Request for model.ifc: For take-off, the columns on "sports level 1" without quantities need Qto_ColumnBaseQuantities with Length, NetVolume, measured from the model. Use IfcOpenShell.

First a look at what the model holds.

```python
import ifcopenshell
import ifcopenshell.util.element
import ifcopenshell.util.unit

model = ifcopenshell.open("model.ifc")
print(model.schema)
for unit_type in ("LENGTHUNIT", "AREAUNIT", "VOLUMEUNIT"):
    print(unit_type, ifcopenshell.util.unit.calculate_unit_scale(model, unit_type))
storey = next(s for s in model.by_type("IfcBuildingStorey") if s.Name == "sports level 1")
columns = [e for e in ifcopenshell.util.element.get_decomposition(storey) if e.is_a("IfcColumn")]
for e in sorted(columns, key=lambda e: e.id()):
    print(e.id(), e.is_a(), e.Name, list(ifcopenshell.util.element.get_psets(e, qtos_only=True)), sep=" | ")
```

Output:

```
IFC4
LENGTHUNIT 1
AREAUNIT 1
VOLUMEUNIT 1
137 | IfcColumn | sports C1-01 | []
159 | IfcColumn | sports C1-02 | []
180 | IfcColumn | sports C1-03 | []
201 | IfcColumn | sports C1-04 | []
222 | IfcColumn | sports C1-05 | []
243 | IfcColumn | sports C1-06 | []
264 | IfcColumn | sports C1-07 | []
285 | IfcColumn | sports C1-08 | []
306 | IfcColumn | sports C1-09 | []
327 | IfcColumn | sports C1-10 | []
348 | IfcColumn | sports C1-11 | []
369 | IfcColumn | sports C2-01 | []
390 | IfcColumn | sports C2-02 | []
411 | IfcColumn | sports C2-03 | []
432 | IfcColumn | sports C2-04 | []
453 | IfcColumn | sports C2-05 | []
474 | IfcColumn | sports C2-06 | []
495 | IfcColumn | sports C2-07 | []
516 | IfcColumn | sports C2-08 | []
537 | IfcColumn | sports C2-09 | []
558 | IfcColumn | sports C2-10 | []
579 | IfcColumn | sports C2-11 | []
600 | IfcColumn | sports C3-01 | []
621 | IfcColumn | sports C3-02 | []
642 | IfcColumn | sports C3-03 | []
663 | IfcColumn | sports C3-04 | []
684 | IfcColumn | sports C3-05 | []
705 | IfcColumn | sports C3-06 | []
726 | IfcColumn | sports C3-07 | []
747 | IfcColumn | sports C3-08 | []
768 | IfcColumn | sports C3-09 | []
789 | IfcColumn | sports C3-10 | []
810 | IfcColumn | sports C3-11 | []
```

```python
import ifcopenshell
import ifcopenshell.api.pset
import ifcopenshell.geom
import ifcopenshell.util.element
import ifcopenshell.util.shape
import ifcopenshell.util.unit

model = ifcopenshell.open("model.ifc")
unit_scale = ifcopenshell.util.unit.calculate_unit_scale(model)
volume_scale = ifcopenshell.util.unit.calculate_unit_scale(model, "VOLUMEUNIT")
settings = ifcopenshell.geom.settings()

storey = next(s for s in model.by_type("IfcBuildingStorey") if s.Name == "sports level 1")
columns = [e for e in ifcopenshell.util.element.get_decomposition(storey) if e.is_a("IfcColumn")]

for e in sorted(columns, key=lambda e: e.id()):
    if ifcopenshell.util.element.get_psets(e, qtos_only=True, should_inherit=False):
        continue
    # Geometry comes back in metres, in the element's own axes.
    shape = ifcopenshell.geom.create_shape(settings, e)
    values = {
        "Length": ifcopenshell.util.shape.get_z(shape.geometry) / unit_scale,
        "NetVolume": ifcopenshell.util.shape.get_volume(shape.geometry) / volume_scale,
    }
    qto = ifcopenshell.api.pset.add_qto(model, product=e, name="Qto_ColumnBaseQuantities")
    ifcopenshell.api.pset.edit_qto(model, qto=qto, properties=values)
    print(e.id(), {k: round(v, 3) for k, v in values.items()})

model.write("model_v2.ifc")
```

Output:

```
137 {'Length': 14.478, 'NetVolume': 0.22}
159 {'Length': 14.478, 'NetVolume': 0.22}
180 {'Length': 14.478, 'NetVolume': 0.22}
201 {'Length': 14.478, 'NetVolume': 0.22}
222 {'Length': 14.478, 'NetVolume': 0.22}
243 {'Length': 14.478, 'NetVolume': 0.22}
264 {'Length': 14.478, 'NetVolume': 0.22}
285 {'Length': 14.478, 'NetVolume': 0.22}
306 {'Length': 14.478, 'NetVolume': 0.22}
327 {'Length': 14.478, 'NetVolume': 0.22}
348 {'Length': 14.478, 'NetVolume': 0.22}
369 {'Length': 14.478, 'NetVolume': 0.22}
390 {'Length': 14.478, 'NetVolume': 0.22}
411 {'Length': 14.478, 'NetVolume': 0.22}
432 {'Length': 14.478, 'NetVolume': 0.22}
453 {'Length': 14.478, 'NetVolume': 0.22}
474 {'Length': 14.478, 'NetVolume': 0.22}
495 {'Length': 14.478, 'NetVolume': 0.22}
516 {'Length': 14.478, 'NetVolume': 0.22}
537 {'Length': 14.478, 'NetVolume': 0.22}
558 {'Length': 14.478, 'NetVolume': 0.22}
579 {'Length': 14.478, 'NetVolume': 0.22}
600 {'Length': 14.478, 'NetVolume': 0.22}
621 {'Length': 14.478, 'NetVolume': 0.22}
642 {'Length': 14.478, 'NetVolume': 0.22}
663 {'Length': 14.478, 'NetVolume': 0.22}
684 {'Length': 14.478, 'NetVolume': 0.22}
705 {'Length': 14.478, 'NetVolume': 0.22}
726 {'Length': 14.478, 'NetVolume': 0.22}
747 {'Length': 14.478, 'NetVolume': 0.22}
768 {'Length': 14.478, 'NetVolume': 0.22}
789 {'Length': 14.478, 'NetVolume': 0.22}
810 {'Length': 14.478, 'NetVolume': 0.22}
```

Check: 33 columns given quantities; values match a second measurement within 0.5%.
